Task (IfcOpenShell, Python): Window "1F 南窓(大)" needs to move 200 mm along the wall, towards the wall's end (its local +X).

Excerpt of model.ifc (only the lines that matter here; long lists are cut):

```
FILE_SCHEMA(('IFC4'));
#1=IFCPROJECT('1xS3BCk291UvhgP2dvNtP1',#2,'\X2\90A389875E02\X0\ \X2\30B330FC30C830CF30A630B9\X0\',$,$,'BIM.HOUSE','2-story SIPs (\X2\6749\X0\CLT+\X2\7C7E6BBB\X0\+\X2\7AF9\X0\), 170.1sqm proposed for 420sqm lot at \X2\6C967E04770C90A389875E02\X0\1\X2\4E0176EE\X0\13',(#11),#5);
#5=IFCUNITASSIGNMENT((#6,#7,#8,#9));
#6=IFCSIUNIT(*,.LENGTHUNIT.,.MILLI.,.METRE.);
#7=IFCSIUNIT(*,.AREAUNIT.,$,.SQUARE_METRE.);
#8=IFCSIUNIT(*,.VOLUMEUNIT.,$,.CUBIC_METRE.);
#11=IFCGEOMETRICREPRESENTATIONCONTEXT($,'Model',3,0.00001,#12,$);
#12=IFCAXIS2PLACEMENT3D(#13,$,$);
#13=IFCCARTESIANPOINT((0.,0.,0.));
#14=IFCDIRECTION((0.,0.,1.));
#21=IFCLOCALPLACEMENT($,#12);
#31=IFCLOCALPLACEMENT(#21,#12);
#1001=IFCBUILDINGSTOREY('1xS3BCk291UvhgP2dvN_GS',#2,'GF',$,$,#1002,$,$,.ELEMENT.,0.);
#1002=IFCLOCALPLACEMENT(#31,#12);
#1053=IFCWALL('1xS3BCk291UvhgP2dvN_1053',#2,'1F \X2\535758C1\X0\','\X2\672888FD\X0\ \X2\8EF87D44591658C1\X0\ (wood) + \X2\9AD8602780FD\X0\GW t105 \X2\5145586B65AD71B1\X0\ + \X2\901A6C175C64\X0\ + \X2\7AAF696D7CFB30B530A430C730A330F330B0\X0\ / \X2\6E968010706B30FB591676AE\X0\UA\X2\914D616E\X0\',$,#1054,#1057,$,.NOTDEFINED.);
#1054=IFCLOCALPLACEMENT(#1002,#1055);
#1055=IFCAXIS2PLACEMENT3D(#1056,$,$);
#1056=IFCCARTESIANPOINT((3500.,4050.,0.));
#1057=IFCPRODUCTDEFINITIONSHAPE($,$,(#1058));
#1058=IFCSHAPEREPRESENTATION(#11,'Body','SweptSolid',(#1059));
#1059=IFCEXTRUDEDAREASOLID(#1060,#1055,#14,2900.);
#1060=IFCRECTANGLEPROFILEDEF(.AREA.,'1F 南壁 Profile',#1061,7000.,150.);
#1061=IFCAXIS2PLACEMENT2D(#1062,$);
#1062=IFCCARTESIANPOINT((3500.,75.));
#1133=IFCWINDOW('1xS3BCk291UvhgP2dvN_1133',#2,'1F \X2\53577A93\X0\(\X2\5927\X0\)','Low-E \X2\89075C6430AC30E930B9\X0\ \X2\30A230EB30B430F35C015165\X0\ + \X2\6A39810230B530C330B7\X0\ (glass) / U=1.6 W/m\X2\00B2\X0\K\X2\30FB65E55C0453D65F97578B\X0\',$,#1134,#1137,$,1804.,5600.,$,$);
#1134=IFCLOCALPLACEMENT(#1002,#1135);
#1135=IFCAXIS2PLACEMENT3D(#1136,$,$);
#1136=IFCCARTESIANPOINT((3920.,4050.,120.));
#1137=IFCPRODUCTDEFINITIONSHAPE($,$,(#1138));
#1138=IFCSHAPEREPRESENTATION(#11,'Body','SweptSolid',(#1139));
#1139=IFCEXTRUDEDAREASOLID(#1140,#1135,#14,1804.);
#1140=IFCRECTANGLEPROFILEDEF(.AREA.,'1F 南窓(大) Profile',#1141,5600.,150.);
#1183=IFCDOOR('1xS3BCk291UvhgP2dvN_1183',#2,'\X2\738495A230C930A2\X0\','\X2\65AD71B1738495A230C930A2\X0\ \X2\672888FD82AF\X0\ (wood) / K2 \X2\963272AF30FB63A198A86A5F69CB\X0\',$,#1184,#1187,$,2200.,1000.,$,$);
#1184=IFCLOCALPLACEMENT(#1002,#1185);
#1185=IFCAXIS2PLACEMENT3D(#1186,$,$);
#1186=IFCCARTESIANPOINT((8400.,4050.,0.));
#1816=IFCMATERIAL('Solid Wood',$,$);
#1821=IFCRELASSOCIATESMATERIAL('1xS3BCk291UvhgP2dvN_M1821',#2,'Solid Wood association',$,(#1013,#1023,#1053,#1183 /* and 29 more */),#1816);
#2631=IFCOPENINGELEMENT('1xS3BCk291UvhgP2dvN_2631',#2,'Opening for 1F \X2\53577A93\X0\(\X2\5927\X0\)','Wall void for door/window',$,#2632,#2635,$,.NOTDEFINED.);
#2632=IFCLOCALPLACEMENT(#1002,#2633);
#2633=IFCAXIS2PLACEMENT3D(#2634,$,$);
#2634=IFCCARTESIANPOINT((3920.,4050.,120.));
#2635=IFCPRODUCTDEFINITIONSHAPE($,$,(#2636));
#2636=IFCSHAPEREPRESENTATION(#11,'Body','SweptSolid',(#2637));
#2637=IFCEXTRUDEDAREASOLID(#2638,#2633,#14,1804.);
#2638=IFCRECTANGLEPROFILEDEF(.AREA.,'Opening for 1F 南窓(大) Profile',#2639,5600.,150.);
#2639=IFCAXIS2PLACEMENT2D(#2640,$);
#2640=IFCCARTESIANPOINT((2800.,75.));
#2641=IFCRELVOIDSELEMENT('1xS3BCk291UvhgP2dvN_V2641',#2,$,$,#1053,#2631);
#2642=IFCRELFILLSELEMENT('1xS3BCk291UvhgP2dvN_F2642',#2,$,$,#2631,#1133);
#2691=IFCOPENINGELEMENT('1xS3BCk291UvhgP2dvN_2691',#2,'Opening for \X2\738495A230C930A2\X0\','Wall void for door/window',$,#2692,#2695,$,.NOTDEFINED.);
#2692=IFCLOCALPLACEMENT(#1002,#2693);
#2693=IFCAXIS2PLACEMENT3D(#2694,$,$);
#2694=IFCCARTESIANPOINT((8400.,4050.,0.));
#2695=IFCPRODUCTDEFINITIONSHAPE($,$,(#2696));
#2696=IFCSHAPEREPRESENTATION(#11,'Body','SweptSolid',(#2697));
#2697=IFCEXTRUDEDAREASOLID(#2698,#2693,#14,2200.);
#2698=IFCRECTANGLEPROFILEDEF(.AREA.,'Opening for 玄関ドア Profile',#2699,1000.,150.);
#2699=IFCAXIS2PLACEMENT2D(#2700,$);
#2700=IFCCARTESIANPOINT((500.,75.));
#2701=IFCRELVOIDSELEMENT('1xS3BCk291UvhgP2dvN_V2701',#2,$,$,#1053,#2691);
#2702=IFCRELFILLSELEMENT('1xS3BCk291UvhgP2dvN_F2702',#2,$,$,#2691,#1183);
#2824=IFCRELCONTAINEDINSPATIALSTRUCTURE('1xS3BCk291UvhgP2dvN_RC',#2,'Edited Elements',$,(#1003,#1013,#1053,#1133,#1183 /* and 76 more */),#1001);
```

```python
import ifcopenshell
import ifcopenshell.api.geometry
import ifcopenshell.util.placement

model = ifcopenshell.open("model.ifc")

window = model.by_guid("1xS3BCk291UvhgP2dvN_1133")
opening = window.FillsVoids[0].RelatingOpeningElement
wall = opening.VoidsElements[0].RelatingBuildingElement

wall_matrix = ifcopenshell.util.placement.get_local_placement(wall.ObjectPlacement)
shift = wall_matrix[:3, 0] * 200.0
before = ifcopenshell.util.placement.get_local_placement(window.ObjectPlacement)[:3, 3].copy()

# The window is not placed relative to its opening, so move both.
for product in (opening, window):
    matrix = ifcopenshell.util.placement.get_local_placement(product.ObjectPlacement)
    matrix[:3, 3] += shift
    ifcopenshell.api.geometry.edit_object_placement(model, product=product, matrix=matrix, is_si=False)

after = ifcopenshell.util.placement.get_local_placement(window.ObjectPlacement)[:3, 3]
print("window moved by", (after - before).round(3) + 0.0)

model.write("model_updated.ifc")
```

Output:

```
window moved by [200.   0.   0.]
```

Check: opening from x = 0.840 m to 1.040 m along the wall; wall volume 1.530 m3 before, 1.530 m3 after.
